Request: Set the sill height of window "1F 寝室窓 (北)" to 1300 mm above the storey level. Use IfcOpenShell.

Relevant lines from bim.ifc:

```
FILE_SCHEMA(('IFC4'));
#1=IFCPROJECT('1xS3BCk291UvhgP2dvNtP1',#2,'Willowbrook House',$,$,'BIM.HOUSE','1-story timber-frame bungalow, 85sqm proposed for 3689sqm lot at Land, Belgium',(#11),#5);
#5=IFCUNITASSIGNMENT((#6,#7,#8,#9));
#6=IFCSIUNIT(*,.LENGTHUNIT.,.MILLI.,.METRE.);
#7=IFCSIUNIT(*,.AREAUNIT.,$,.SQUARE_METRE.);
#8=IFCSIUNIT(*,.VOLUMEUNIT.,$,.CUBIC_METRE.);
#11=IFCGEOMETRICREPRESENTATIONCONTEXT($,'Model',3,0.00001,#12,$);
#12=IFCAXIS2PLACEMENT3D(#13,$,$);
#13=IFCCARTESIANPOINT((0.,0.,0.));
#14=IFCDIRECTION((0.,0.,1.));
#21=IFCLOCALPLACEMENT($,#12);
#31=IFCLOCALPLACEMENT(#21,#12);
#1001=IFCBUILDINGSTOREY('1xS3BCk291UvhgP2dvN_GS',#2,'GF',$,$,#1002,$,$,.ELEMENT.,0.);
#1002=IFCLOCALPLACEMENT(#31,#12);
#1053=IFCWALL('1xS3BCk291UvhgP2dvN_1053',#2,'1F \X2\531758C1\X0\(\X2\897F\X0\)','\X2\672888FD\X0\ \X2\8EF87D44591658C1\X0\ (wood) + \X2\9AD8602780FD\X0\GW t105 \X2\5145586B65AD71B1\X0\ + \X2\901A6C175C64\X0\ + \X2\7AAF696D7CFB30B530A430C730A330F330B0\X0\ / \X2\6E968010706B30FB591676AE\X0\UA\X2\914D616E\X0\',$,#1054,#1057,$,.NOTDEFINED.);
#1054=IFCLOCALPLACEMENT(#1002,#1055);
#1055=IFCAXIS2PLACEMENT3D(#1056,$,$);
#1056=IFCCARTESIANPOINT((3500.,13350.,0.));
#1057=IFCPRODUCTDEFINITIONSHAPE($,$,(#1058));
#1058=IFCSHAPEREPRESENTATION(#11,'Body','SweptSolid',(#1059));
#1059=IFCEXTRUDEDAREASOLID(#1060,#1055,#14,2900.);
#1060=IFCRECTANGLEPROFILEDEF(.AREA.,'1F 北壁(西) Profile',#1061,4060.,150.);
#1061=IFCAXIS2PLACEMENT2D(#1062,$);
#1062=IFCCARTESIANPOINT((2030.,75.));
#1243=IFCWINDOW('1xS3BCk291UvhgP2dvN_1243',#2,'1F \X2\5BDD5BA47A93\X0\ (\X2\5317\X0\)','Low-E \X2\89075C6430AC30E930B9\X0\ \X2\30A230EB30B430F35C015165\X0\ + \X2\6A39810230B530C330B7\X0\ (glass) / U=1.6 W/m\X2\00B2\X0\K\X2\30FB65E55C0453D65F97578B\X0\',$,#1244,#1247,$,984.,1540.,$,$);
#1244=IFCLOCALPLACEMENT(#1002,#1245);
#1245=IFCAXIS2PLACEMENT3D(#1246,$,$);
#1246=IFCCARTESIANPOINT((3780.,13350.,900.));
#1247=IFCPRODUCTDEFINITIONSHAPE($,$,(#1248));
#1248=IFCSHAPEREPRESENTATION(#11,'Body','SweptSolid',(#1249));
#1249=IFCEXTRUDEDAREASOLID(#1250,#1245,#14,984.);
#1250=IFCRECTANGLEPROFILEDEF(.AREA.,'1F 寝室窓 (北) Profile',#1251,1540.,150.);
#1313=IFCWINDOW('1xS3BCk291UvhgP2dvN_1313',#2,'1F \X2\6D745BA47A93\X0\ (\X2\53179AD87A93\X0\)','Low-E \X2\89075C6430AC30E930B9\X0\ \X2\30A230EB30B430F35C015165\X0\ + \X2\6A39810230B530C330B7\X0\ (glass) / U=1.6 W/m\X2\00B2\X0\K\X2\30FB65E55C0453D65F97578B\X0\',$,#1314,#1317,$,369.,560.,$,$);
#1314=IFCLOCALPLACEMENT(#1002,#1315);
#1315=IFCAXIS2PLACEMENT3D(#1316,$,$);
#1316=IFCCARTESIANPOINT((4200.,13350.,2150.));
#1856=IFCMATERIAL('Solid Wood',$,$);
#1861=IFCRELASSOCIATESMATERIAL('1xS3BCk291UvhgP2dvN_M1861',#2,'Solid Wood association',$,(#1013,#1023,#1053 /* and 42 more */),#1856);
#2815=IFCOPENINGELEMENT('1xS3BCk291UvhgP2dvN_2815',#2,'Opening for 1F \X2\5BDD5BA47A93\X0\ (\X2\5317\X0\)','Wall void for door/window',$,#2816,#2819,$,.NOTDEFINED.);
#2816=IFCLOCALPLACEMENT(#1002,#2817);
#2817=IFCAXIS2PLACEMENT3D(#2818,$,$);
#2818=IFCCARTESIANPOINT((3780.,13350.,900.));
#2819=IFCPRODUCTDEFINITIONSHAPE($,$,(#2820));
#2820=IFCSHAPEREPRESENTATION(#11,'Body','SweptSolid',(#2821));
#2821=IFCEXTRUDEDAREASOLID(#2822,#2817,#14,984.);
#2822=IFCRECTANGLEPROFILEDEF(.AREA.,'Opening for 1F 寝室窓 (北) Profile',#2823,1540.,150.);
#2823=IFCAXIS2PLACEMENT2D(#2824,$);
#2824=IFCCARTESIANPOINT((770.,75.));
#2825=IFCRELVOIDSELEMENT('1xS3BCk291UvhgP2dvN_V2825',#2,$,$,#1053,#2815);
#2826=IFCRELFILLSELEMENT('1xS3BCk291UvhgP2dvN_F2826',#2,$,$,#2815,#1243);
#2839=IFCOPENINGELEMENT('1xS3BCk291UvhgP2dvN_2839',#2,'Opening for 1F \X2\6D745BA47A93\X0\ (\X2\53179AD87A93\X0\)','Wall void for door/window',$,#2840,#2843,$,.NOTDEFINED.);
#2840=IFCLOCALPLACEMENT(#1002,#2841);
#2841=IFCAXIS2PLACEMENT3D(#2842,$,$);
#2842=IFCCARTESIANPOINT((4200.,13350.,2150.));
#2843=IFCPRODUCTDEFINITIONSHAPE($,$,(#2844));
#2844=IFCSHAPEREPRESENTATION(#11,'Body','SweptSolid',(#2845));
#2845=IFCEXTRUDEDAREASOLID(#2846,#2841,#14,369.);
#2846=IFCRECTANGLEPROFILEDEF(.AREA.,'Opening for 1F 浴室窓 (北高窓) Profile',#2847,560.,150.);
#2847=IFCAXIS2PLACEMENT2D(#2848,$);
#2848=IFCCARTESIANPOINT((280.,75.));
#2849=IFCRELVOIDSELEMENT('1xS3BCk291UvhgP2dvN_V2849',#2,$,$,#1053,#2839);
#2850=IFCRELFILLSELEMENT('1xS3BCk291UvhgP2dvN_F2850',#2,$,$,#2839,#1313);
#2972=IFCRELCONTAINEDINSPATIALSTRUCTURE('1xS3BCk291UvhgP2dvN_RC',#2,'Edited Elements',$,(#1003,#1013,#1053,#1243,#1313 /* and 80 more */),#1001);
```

```python
import numpy as np
import ifcopenshell
import ifcopenshell.api.geometry
import ifcopenshell.geom
import ifcopenshell.util.element
import ifcopenshell.util.placement
import ifcopenshell.util.shape
import ifcopenshell.util.unit

model = ifcopenshell.open("bim.ifc")
unit_scale = ifcopenshell.util.unit.calculate_unit_scale(model)

window = model.by_id(1243)
opening = window.FillsVoids[0].RelatingOpeningElement
storey = ifcopenshell.util.element.get_container(window, ifc_class="IfcBuildingStorey")
level = ifcopenshell.util.placement.get_local_placement(storey.ObjectPlacement)[2, 3]

# The opening's origin need not be at the sill, so measure its lowest point.
shape = ifcopenshell.geom.create_shape(ifcopenshell.geom.settings(), opening)
bottom = ifcopenshell.util.shape.get_shape_bottom_elevation(shape, shape.geometry) / unit_scale
dz = level + 1.3 / unit_scale - bottom

shift = np.array([0.0, 0.0, dz])
# The window is not placed relative to its opening, so move both.
for product in (opening, window):
    matrix = ifcopenshell.util.placement.get_local_placement(product.ObjectPlacement)
    matrix[:3, 3] += shift
    ifcopenshell.api.geometry.edit_object_placement(model, product=product, matrix=matrix, is_si=False)

print(f"moved by {dz * unit_scale:+.3f} m")

model.write("bim_updated.ifc")
```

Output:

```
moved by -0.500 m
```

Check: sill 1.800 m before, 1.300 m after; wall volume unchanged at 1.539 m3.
